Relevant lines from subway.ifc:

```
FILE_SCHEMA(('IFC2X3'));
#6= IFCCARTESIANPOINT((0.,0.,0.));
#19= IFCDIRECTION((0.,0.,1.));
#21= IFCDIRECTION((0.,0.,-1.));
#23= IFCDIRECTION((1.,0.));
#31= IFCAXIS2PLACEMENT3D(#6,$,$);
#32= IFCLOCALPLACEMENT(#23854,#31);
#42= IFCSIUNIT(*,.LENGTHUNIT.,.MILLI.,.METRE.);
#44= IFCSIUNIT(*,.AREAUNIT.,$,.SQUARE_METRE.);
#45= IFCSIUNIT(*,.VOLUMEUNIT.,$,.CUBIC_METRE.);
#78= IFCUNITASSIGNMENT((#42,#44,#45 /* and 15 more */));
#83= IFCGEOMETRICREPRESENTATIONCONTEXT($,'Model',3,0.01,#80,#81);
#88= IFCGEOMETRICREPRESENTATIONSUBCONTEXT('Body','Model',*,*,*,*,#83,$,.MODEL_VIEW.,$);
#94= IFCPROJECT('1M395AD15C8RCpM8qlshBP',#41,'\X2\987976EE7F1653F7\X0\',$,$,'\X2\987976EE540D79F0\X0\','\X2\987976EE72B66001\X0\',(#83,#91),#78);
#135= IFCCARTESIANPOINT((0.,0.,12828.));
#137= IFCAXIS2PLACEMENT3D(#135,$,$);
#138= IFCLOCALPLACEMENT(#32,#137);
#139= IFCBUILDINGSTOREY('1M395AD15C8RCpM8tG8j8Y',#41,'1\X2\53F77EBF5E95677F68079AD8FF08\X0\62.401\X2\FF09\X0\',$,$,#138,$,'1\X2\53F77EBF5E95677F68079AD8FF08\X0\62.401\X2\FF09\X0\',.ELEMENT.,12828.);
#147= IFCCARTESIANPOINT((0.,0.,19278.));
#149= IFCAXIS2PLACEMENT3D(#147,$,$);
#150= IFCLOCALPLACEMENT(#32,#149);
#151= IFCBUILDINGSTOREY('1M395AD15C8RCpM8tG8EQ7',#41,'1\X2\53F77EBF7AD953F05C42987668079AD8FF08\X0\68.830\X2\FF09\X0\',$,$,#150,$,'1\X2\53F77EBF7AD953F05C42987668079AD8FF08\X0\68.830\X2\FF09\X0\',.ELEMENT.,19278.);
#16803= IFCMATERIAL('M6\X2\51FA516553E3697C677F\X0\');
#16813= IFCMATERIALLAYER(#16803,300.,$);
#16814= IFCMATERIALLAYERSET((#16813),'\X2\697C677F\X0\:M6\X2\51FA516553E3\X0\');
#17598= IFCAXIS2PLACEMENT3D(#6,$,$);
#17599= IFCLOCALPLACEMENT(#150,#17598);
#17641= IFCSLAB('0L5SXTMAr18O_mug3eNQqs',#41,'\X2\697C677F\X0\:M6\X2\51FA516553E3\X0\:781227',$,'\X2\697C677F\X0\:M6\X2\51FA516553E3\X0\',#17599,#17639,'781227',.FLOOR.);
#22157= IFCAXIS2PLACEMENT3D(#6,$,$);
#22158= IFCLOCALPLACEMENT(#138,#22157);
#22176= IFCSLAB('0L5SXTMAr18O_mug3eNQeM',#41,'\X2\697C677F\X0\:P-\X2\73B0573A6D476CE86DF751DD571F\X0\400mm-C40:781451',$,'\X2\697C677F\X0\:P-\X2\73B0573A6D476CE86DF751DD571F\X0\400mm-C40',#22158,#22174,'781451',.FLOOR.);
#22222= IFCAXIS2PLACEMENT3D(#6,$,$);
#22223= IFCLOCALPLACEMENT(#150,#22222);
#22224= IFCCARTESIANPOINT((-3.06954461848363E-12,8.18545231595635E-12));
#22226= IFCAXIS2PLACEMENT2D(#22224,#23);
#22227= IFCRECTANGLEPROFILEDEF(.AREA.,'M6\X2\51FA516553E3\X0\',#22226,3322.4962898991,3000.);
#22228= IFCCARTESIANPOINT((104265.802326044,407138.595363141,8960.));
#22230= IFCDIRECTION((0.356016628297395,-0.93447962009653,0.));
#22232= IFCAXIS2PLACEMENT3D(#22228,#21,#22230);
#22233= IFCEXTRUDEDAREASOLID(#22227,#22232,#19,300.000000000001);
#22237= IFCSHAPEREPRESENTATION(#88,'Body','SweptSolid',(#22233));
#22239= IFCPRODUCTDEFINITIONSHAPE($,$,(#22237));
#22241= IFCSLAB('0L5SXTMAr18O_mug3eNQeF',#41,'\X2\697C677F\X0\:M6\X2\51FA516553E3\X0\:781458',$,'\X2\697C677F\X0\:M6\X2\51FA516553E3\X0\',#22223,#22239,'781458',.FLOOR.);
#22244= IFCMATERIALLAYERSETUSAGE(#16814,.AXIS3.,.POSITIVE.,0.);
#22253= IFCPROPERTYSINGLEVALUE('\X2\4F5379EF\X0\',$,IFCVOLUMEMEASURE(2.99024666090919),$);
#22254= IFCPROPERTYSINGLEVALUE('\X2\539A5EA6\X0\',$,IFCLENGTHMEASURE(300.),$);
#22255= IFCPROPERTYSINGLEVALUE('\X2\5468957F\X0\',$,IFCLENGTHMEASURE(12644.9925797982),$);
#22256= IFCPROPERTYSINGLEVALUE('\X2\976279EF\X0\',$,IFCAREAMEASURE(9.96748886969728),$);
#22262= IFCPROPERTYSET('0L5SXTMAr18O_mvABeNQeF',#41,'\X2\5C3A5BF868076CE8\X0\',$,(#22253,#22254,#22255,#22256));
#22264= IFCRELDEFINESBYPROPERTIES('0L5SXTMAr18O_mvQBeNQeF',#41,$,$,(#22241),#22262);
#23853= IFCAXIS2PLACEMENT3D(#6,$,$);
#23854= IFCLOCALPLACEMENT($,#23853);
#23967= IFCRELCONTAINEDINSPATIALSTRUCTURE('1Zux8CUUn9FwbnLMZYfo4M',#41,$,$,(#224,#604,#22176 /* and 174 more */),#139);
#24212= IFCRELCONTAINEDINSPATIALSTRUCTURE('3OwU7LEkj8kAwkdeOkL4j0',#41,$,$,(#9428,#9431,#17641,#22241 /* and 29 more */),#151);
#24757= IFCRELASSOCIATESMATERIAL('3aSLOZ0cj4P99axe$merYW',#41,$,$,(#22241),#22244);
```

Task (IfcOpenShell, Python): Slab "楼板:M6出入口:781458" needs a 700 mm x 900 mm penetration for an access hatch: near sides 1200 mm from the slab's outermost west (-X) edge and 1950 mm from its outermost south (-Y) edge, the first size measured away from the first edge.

```python
import numpy as np
import ifcopenshell
import ifcopenshell.api.feature
import ifcopenshell.api.geometry
import ifcopenshell.api.pset
import ifcopenshell.api.root
import ifcopenshell.geom
import ifcopenshell.util.element
import ifcopenshell.util.placement
import ifcopenshell.util.representation
import ifcopenshell.util.shape
import ifcopenshell.util.unit

model = ifcopenshell.open("subway.ifc")
unit_scale = ifcopenshell.util.unit.calculate_unit_scale(model)
area_scale = ifcopenshell.util.unit.calculate_unit_scale(model, "AREAUNIT")
volume_scale = ifcopenshell.util.unit.calculate_unit_scale(model, "VOLUMEUNIT")
settings = ifcopenshell.geom.settings()


def volume(element):
    """Net volume in cubic metres, openings subtracted."""
    shape = ifcopenshell.geom.create_shape(settings, element)
    return ifcopenshell.util.shape.get_volume(shape.geometry)


slab = model.by_guid("0L5SXTMAr18O_mug3eNQeF")
before = volume(slab)

# Extent in the slab's own axes, in metres. The edges named are its -X and -Y sides.
slab_shape = ifcopenshell.geom.create_shape(settings, slab)
vertices = ifcopenshell.util.shape.get_vertices(slab_shape.geometry)
x_min, y_min, bottom = vertices.min(axis=0)
top = vertices[:, 2].max()

opening = ifcopenshell.api.root.create_entity(model, ifc_class="IfcOpeningElement", name="Access hatch opening")
context = ifcopenshell.util.representation.get_context(model, "Model", "Body", "MODEL_VIEW")
width, depth = 0.7, 0.9
outline = [(0.0, 0.0), (width, 0.0), (width, depth), (0.0, depth), (0.0, 0.0)]
# Overshoot both faces by 50 mm so the cut is clean.
shape = ifcopenshell.api.geometry.add_slab_representation(
    model, context=context, depth=top - bottom + 0.1, polyline=outline
)
ifcopenshell.api.geometry.assign_representation(model, product=opening, representation=shape)

matrix = ifcopenshell.util.placement.get_local_placement(slab.ObjectPlacement)
matrix[:, 3] = matrix @ np.append(np.array([x_min + 1.2, y_min + 1.95, bottom - 0.05]) / unit_scale, 1.0)
ifcopenshell.api.geometry.edit_object_placement(model, product=opening, matrix=matrix, is_si=False)
ifcopenshell.api.feature.add_feature(model, feature=opening, element=slab)

after = volume(slab)

# Update the slab's stored quantities.
pset = model.by_id(ifcopenshell.util.element.get_pset(slab, "尺寸标注", should_inherit=False)["id"])
ifcopenshell.api.pset.edit_pset(model, pset=pset, properties={
    "体积": model.create_entity("IfcVolumeMeasure", after / volume_scale),
    "面积": model.create_entity("IfcAreaMeasure", after / (top - bottom) / area_scale),
})

print(f"slab volume {before:.3f} -> {after:.3f} m3")

model.write("subway_edited.ifc")
```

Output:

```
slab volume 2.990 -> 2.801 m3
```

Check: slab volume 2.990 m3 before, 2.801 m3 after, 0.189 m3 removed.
